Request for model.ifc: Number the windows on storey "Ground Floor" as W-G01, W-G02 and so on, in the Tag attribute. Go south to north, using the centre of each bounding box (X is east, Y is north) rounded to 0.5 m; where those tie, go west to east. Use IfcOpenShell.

First a look at what the model holds.

```python
import ifcopenshell
import ifcopenshell.util.element
import ifcopenshell.util.placement

model = ifcopenshell.open("model.ifc")
print(model.schema)
storey = next(s for s in model.by_type("IfcBuildingStorey") if s.Name == "Ground Floor")
windows = [e for e in ifcopenshell.util.element.get_decomposition(storey) if e.is_a("IfcWindow")]
for e in sorted(windows, key=lambda e: e.id()):
    origin = ifcopenshell.util.placement.get_local_placement(e.ObjectPlacement)[:3, 3]
    print(e.id(), e.Tag, e.Name, origin.round(2) + 0.0, sep=" | ")
```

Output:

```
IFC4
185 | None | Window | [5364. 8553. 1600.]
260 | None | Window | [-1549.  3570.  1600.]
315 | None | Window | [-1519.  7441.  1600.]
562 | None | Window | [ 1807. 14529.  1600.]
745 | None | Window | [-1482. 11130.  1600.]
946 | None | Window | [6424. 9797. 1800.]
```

```python
import ifcopenshell
import ifcopenshell.geom
import ifcopenshell.util.element
import ifcopenshell.util.shape

model = ifcopenshell.open("model.ifc")
settings = ifcopenshell.geom.settings()
settings.set("use-world-coords", True)


def centre(element):
    shape = ifcopenshell.geom.create_shape(settings, element)
    return ifcopenshell.util.shape.get_bbox_centroid(shape.geometry)


storey = next(s for s in model.by_type("IfcBuildingStorey") if s.Name == "Ground Floor")
windows = [e for e in ifcopenshell.util.element.get_decomposition(storey) if e.is_a("IfcWindow")]

# Insertion points can sit at a corner or the storey origin, so sort by the geometry (in metres).
centres = {e: centre(e) for e in windows}
windows.sort(key=lambda e: (round(centres[e][1] / 0.5), centres[e][0]))

for i, e in enumerate(windows, start=1):
    number = f"W-G{i:02d}"
    e.Tag = number
    print(e.id(), number)

model.write("model_updated.ifc")
```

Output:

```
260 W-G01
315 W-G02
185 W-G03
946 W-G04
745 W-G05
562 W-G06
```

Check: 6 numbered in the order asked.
